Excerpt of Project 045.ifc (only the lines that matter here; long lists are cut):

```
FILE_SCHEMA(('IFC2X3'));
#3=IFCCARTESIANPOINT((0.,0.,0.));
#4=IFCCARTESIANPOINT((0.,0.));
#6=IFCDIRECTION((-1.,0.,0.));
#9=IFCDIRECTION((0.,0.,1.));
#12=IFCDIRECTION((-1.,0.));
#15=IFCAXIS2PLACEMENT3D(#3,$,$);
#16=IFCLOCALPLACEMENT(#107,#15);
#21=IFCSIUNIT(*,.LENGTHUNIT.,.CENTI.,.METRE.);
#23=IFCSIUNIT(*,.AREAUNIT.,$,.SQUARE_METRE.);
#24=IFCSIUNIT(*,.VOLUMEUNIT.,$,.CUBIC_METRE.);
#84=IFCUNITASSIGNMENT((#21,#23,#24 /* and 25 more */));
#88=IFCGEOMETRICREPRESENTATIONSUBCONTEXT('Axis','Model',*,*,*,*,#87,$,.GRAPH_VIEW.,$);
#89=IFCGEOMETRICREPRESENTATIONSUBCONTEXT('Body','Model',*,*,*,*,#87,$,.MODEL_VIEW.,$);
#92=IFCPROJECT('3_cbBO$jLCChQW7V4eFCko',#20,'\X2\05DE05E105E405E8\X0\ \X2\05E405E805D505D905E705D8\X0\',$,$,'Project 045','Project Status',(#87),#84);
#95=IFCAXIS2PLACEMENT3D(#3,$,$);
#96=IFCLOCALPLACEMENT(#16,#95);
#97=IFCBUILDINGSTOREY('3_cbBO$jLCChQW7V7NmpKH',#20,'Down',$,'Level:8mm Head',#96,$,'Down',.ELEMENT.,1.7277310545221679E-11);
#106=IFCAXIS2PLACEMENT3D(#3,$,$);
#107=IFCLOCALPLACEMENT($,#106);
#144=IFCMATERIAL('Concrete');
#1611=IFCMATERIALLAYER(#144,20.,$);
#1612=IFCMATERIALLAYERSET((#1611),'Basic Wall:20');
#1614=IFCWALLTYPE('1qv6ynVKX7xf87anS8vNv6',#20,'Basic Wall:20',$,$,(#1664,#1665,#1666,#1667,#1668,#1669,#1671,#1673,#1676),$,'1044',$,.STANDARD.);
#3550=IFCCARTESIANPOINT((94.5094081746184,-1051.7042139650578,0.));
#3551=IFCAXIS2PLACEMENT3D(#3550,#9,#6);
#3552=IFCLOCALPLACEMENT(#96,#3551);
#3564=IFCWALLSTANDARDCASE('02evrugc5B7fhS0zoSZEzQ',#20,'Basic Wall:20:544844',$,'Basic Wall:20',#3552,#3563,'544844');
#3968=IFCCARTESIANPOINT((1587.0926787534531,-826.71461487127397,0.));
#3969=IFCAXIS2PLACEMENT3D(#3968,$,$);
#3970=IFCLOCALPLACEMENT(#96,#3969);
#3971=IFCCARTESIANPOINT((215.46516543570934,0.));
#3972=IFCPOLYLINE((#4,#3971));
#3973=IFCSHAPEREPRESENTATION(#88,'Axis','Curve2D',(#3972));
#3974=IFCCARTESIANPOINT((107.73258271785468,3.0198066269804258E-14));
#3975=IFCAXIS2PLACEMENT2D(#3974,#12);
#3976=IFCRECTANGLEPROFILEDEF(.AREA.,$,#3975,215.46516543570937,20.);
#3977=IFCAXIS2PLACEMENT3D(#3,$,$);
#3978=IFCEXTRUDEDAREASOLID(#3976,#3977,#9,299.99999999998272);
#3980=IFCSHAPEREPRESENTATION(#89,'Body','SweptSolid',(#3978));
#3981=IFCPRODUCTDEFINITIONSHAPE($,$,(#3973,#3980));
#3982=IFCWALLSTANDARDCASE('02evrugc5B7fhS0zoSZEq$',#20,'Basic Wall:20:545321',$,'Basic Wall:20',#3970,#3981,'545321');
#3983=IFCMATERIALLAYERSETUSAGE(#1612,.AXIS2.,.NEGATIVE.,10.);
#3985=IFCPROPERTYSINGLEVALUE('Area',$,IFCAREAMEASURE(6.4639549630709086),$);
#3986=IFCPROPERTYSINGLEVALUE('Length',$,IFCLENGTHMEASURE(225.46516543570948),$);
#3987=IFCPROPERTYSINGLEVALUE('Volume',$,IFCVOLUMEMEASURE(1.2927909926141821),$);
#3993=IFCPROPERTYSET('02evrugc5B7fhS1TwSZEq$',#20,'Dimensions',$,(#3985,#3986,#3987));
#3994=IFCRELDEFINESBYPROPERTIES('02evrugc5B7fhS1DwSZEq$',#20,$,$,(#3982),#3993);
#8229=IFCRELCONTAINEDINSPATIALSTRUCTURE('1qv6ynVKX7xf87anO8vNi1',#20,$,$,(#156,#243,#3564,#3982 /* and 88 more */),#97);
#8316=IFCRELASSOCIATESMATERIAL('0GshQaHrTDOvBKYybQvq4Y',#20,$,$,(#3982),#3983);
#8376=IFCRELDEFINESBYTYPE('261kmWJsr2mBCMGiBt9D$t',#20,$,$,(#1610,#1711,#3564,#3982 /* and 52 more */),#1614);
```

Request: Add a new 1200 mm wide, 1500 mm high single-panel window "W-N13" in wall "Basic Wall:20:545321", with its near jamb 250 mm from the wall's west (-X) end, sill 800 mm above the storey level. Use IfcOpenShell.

```python
import numpy as np
import ifcopenshell
import ifcopenshell.api.feature
import ifcopenshell.api.geometry
import ifcopenshell.api.pset
import ifcopenshell.api.root
import ifcopenshell.api.spatial
import ifcopenshell.api.type
import ifcopenshell.geom
import ifcopenshell.util.element
import ifcopenshell.util.placement
import ifcopenshell.util.representation
import ifcopenshell.util.shape
import ifcopenshell.util.unit

model = ifcopenshell.open("Project 045.ifc")
unit_scale = ifcopenshell.util.unit.calculate_unit_scale(model)
area_scale = ifcopenshell.util.unit.calculate_unit_scale(model, "AREAUNIT")
volume_scale = ifcopenshell.util.unit.calculate_unit_scale(model, "VOLUMEUNIT")
settings = ifcopenshell.geom.settings()


def volume(element):
    """Net volume in cubic metres, openings subtracted."""
    shape = ifcopenshell.geom.create_shape(settings, element)
    return ifcopenshell.util.shape.get_volume(shape.geometry)


wall = model.by_guid("02evrugc5B7fhS0zoSZEq$")
storey = ifcopenshell.util.element.get_container(wall, ifc_class="IfcBuildingStorey")
context = ifcopenshell.util.representation.get_context(model, "Model", "Body", "MODEL_VIEW")
before = volume(wall)

width, height, from_end, sill = 1.2, 1.5, 0.25, 0.8  # metres

# The wall runs along its own X axis, and the end named is its -X end.
wall_shape = ifcopenshell.geom.create_shape(settings, wall)
x, y, z = ifcopenshell.util.shape.get_vertices(wall_shape.geometry).T
start = x.min() + from_end
face, thickness = float(y.min()), float(y.max() - y.min())
wall_matrix = ifcopenshell.util.placement.get_local_placement(wall.ObjectPlacement)
level = ifcopenshell.util.placement.get_local_placement(storey.ObjectPlacement)[2, 3]


def in_wall(x, y):
    """Placement at x, y metres in the wall's axes, at sill height."""
    matrix = wall_matrix.copy()
    matrix[:, 3] = wall_matrix @ np.array([x / unit_scale, y / unit_scale, 0.0, 1.0])
    matrix[2, 3] = level + sill / unit_scale
    return matrix


# Opening: a box that overshoots both wall faces by 50 mm.
opening = ifcopenshell.api.root.create_entity(model, ifc_class="IfcOpeningElement")
box = ifcopenshell.api.geometry.add_wall_representation(
    model, context=context, length=width, height=height, thickness=thickness + 0.1
)
ifcopenshell.api.geometry.assign_representation(model, product=opening, representation=box)
ifcopenshell.api.geometry.edit_object_placement(model, product=opening, matrix=in_wall(start, face - 0.05), is_si=False)
ifcopenshell.api.feature.add_feature(model, feature=opening, element=wall)

window = ifcopenshell.api.root.create_entity(model, ifc_class="IfcWindow", name="W-N13")
window.OverallWidth, window.OverallHeight = width / unit_scale, height / unit_scale
body = ifcopenshell.api.geometry.add_window_representation(
    model,
    context=context,
    overall_width=window.OverallWidth,
    overall_height=window.OverallHeight,
    partition_type="SINGLE_PANEL",
)
ifcopenshell.api.geometry.assign_representation(model, product=window, representation=body)
ifcopenshell.api.spatial.assign_container(model, products=[window], relating_structure=storey)
fills = ifcopenshell.api.feature.add_filling(model, opening=opening, element=window)
fills.OwnerHistory = window.OwnerHistory  # required in IFC2X3

# IFC2X3 keeps the operation on the window style.
style = ifcopenshell.api.root.create_entity(model, ifc_class="IfcWindowStyle", name="W-N13")
style.OperationType, style.ConstructionType = "SINGLE_PANEL", "NOTDEFINED"
style.ParameterTakesPrecedence = style.Sizeable = False
ifcopenshell.api.type.assign_type(model, related_objects=[window], relating_type=style)

# Centre the window in the wall's thickness.
ifcopenshell.api.geometry.edit_object_placement(model, product=window, matrix=in_wall(start, face), is_si=False)
window_shape = ifcopenshell.geom.create_shape(settings, window)
depth = ifcopenshell.util.shape.get_vertices(window_shape.geometry)[:, 1]
offset = face + thickness / 2 - (depth.min() + depth.max()) / 2
ifcopenshell.api.geometry.edit_object_placement(model, product=window, matrix=in_wall(start, offset), is_si=False)

after = volume(wall)

# Update the wall's stored quantities.
pset = model.by_id(ifcopenshell.util.element.get_pset(wall, "Dimensions", should_inherit=False)["id"])
ifcopenshell.api.pset.edit_pset(model, pset=pset, properties={
    "Area": model.create_entity("IfcAreaMeasure", after / thickness / area_scale),
    "Volume": model.create_entity("IfcVolumeMeasure", after / volume_scale),
})

print(f"wall volume {before:.3f} -> {after:.3f} m3")

model.write("Project 045_v2.ifc")
```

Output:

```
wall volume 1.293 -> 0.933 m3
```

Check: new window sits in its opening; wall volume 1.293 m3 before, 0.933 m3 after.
